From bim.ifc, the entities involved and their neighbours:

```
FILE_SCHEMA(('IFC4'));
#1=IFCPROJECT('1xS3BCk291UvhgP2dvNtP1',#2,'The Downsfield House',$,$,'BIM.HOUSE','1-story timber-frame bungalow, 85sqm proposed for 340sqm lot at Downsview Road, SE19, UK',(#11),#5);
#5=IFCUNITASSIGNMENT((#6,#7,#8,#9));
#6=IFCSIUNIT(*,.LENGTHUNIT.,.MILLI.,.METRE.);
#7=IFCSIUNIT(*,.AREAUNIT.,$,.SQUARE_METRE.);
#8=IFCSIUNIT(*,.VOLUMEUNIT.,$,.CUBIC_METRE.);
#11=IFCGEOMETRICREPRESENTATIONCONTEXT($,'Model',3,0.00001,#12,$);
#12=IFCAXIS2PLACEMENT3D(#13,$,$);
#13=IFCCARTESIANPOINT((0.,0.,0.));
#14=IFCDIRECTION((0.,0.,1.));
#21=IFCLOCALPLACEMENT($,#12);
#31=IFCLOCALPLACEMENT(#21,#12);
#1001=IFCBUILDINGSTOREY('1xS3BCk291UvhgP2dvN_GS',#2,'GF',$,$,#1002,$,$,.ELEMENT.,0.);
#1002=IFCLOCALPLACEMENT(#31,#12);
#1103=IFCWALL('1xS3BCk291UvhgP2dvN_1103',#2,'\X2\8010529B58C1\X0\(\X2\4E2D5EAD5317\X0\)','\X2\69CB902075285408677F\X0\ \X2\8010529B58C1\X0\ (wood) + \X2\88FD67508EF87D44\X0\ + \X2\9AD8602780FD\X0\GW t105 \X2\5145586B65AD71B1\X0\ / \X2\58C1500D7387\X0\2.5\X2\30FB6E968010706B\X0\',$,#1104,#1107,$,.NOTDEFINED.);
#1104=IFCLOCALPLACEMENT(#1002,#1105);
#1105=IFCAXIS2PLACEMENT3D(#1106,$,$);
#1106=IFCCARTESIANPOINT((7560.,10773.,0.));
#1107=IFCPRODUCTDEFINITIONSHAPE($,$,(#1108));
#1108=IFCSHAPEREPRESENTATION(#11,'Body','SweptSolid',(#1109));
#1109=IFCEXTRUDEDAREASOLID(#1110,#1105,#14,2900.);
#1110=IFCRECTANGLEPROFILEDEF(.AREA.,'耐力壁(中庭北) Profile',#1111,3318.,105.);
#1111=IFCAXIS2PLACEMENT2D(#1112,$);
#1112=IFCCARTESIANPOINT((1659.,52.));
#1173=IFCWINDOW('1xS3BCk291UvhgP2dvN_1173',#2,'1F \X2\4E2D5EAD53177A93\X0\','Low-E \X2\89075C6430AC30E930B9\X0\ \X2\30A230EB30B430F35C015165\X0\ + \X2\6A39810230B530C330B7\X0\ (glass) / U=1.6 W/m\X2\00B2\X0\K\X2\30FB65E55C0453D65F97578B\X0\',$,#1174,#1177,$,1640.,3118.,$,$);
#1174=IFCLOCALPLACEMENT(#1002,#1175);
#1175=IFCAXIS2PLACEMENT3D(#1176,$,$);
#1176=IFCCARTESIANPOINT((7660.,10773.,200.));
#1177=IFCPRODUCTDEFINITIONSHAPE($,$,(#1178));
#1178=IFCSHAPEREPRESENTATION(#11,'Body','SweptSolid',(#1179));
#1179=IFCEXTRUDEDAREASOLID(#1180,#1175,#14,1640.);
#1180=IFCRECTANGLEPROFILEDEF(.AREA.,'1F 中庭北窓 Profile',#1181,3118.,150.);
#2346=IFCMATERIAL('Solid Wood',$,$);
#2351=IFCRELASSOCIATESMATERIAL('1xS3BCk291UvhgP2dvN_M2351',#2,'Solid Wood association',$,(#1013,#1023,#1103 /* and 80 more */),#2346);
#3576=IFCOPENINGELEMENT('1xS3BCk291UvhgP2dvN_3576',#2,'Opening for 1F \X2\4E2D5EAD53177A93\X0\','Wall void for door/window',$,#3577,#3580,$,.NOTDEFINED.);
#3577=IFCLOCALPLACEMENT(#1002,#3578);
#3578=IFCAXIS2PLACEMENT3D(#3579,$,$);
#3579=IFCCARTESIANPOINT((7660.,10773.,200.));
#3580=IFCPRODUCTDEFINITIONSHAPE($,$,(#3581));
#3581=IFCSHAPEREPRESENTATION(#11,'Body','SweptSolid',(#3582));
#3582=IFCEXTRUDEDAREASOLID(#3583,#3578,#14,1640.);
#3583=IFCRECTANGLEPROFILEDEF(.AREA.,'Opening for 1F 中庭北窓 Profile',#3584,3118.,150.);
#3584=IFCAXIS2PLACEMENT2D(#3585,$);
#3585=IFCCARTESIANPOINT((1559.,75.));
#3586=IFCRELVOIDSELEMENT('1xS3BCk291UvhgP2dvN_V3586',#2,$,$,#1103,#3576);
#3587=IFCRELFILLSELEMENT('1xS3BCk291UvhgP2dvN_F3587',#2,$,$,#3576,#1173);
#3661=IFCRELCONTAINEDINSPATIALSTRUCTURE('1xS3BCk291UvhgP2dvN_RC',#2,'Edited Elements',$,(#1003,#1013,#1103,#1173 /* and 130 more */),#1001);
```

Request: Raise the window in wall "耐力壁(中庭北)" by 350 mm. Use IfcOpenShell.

```python
import numpy as np
import ifcopenshell
import ifcopenshell.api.geometry
import ifcopenshell.util.placement
import ifcopenshell.util.unit

model = ifcopenshell.open("bim.ifc")
unit_scale = ifcopenshell.util.unit.calculate_unit_scale(model)

window = model.by_id(1173)
opening = window.FillsVoids[0].RelatingOpeningElement
dz = 0.35 / unit_scale

shift = np.array([0.0, 0.0, dz])
# The window is not placed relative to its opening, so move both.
for product in (opening, window):
    matrix = ifcopenshell.util.placement.get_local_placement(product.ObjectPlacement)
    matrix[:3, 3] += shift
    ifcopenshell.api.geometry.edit_object_placement(model, product=product, matrix=matrix, is_si=False)

print(f"moved by {dz * unit_scale:+.3f} m")

model.write("bim_v2.ifc")
```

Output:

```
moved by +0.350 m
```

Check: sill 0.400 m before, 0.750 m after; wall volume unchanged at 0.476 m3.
